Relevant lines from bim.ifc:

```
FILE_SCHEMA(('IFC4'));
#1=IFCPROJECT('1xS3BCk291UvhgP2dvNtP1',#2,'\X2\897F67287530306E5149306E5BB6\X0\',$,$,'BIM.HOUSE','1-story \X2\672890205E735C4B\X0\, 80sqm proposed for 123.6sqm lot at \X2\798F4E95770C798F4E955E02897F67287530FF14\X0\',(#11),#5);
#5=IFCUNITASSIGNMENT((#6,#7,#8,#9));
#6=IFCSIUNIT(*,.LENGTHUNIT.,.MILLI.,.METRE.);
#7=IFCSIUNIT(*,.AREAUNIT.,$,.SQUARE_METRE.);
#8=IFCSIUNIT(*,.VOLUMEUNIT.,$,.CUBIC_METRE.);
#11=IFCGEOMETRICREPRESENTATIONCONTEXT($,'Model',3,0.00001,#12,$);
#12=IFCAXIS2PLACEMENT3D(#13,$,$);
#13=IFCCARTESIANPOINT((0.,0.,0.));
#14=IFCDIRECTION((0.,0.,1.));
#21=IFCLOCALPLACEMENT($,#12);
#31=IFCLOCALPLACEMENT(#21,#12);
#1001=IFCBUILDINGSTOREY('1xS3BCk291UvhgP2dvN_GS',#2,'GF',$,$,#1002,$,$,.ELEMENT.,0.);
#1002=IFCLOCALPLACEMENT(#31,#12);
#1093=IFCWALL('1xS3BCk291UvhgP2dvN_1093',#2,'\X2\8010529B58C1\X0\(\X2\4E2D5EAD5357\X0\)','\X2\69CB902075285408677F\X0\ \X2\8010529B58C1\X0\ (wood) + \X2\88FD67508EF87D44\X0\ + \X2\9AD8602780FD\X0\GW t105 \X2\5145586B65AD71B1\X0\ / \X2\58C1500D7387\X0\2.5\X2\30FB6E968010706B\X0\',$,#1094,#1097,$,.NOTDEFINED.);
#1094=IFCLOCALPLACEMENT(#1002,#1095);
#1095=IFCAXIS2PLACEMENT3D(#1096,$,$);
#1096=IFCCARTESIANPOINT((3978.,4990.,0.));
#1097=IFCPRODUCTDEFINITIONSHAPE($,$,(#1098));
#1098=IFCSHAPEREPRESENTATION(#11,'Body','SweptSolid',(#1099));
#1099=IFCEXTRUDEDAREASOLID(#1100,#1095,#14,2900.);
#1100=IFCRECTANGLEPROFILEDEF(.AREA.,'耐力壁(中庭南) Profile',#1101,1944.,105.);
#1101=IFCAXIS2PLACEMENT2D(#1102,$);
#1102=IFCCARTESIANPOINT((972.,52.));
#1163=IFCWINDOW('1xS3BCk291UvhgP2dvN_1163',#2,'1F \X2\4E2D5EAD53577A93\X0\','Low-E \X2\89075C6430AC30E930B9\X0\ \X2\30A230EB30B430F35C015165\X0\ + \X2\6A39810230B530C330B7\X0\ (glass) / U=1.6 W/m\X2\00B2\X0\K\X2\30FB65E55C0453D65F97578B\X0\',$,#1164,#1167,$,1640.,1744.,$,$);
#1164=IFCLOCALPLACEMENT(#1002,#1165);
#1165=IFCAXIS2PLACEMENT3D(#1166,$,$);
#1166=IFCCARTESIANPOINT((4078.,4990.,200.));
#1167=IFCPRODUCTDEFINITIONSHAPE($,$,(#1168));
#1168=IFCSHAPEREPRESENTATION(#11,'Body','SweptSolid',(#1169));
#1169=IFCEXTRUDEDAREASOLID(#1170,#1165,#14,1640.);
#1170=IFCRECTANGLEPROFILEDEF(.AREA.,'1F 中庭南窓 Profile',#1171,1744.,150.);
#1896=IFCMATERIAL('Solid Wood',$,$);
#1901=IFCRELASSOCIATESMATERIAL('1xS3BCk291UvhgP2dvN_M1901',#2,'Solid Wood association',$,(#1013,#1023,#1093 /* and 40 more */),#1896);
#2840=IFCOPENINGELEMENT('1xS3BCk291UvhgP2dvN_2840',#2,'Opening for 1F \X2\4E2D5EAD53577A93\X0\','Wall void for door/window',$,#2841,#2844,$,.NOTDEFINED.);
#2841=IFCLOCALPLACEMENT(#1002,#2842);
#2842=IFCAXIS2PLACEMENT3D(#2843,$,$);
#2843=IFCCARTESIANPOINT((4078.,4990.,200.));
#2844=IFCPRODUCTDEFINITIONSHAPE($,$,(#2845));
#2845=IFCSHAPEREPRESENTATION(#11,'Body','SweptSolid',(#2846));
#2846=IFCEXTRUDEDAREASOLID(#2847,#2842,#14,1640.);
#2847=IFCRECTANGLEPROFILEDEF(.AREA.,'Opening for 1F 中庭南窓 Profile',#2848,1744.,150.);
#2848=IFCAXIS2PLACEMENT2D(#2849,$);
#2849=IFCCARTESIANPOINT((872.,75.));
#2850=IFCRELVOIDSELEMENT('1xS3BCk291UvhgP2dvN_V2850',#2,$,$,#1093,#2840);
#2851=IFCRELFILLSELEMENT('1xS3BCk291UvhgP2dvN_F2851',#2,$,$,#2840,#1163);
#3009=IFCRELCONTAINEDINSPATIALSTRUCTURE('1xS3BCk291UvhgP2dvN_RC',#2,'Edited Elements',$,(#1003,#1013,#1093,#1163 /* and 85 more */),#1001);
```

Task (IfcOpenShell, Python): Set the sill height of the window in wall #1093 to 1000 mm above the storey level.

```python
import numpy as np
import ifcopenshell
import ifcopenshell.api.geometry
import ifcopenshell.geom
import ifcopenshell.util.element
import ifcopenshell.util.placement
import ifcopenshell.util.shape
import ifcopenshell.util.unit

model = ifcopenshell.open("bim.ifc")
unit_scale = ifcopenshell.util.unit.calculate_unit_scale(model)

window = model.by_guid("1xS3BCk291UvhgP2dvN_1163")
opening = window.FillsVoids[0].RelatingOpeningElement
storey = ifcopenshell.util.element.get_container(window, ifc_class="IfcBuildingStorey")
level = ifcopenshell.util.placement.get_local_placement(storey.ObjectPlacement)[2, 3]

# The opening's origin need not be at the sill, so measure its lowest point.
shape = ifcopenshell.geom.create_shape(ifcopenshell.geom.settings(), opening)
bottom = ifcopenshell.util.shape.get_shape_bottom_elevation(shape, shape.geometry) / unit_scale
dz = level + 1000.0 - bottom

shift = np.array([0.0, 0.0, dz])
# The window is not placed relative to its opening, so move both.
for product in (opening, window):
    matrix = ifcopenshell.util.placement.get_local_placement(product.ObjectPlacement)
    matrix[:3, 3] += shift
    ifcopenshell.api.geometry.edit_object_placement(model, product=product, matrix=matrix, is_si=False)

print(f"moved by {dz * unit_scale:+.3f} m")

model.write("bim_edited.ifc")
```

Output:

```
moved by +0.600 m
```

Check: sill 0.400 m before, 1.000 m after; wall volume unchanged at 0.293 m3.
